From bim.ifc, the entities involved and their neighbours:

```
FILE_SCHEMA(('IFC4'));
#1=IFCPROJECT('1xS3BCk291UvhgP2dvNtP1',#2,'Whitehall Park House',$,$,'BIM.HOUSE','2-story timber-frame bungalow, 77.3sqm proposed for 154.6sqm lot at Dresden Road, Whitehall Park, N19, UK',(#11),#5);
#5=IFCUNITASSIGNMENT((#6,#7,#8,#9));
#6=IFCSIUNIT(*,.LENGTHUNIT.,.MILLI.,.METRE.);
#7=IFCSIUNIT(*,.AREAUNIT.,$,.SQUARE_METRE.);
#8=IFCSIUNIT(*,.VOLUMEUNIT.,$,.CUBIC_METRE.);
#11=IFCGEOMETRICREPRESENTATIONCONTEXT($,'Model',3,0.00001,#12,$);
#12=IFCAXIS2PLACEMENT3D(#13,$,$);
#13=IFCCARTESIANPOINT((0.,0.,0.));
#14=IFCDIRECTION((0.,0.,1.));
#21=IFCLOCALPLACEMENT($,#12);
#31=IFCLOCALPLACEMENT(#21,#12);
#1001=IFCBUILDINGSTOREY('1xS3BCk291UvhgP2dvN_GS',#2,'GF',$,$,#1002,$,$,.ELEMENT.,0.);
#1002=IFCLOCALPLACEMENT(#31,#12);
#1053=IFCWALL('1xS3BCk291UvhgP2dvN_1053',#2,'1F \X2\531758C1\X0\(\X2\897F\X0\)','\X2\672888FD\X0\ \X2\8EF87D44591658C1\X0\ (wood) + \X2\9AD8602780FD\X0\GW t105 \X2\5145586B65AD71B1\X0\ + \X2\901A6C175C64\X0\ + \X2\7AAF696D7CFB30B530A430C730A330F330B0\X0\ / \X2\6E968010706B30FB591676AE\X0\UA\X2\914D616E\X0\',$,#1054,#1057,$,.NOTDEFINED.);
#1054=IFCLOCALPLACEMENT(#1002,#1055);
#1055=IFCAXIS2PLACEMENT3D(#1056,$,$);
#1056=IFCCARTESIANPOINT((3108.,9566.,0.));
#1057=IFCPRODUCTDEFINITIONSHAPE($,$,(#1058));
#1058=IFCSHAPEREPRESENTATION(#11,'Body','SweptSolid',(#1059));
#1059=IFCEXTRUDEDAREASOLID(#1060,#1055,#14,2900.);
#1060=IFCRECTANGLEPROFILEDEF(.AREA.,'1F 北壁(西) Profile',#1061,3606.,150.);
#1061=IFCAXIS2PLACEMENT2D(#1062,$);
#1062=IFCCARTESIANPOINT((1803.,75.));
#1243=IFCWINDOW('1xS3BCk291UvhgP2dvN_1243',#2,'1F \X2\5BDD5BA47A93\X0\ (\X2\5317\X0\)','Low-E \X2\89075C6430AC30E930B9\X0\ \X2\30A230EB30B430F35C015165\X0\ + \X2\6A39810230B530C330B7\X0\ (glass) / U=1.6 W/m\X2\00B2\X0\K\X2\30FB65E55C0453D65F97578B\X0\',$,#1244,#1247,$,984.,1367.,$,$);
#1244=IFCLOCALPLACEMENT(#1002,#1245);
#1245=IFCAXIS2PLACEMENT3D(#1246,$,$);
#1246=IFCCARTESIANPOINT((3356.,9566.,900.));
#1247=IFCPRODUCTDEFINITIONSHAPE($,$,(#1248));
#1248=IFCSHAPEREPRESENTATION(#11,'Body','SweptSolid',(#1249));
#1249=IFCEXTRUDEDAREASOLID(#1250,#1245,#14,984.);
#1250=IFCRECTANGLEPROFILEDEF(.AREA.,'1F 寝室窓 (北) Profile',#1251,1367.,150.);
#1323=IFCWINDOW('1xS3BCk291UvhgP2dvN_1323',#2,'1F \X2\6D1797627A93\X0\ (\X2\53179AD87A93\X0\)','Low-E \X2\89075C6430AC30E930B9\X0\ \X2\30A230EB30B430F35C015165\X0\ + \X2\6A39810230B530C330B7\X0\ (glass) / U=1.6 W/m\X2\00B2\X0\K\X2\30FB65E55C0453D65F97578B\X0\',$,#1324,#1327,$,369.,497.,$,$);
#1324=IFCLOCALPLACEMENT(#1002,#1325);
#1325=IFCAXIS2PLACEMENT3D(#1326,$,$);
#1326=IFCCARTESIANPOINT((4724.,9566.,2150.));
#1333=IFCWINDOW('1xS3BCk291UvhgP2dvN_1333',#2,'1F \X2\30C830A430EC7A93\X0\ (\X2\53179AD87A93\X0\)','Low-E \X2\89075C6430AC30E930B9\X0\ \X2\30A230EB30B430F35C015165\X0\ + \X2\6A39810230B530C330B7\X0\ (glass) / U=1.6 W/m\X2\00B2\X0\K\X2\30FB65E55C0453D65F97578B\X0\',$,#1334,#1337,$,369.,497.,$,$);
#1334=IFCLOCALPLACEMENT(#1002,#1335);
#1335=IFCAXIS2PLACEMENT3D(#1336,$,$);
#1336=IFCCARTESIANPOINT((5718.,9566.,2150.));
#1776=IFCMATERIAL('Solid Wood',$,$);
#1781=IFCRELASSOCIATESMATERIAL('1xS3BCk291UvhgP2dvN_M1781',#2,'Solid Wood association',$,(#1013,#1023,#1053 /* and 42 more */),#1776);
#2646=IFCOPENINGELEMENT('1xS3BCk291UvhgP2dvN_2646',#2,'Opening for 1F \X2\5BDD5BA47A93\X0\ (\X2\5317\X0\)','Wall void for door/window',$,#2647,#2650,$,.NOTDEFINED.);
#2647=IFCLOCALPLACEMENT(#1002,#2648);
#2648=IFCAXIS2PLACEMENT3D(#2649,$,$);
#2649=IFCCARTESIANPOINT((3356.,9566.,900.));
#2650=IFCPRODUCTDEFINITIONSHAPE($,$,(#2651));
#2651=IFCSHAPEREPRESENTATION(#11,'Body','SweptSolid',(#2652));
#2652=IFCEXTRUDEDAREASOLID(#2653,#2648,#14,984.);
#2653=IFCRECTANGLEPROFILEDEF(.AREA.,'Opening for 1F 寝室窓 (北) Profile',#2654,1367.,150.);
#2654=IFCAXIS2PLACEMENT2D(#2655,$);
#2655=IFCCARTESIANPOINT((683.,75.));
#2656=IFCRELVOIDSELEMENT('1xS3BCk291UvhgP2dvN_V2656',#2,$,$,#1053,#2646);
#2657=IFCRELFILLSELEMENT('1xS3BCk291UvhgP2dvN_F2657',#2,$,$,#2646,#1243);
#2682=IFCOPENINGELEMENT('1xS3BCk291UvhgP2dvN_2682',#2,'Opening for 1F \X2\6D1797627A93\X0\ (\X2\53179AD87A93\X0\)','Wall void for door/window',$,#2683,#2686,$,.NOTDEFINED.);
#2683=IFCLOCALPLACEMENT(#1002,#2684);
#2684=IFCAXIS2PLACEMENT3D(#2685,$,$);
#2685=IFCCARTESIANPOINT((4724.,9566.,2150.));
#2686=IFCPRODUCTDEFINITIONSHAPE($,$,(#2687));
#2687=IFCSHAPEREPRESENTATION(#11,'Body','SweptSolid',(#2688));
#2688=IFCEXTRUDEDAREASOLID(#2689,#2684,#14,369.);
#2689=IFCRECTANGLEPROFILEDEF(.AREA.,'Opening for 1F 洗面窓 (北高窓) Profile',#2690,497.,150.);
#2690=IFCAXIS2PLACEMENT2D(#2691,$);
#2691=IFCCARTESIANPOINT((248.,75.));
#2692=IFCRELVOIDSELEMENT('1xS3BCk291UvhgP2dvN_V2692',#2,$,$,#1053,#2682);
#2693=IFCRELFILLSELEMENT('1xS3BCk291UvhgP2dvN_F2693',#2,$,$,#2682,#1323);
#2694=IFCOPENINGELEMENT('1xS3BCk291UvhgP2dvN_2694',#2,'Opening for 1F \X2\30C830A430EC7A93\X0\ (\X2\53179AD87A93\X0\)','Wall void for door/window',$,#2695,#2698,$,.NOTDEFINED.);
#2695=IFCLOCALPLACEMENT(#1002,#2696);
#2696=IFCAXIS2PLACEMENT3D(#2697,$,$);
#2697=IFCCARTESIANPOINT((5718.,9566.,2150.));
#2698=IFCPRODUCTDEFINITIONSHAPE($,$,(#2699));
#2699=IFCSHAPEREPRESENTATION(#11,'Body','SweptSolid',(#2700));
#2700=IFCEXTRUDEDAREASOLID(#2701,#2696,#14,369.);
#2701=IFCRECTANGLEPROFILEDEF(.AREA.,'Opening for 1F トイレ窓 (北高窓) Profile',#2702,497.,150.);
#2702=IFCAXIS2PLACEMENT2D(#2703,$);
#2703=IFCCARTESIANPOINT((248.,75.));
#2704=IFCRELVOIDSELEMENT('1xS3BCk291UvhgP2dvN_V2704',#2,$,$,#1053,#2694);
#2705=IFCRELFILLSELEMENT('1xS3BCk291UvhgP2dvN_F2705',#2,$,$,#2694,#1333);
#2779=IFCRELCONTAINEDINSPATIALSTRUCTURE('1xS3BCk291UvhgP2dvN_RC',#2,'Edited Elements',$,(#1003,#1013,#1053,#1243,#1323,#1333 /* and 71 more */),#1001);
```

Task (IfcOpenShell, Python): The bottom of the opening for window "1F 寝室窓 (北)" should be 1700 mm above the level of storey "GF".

```python
import numpy as np
import ifcopenshell
import ifcopenshell.api.geometry
import ifcopenshell.geom
import ifcopenshell.util.element
import ifcopenshell.util.placement
import ifcopenshell.util.shape
import ifcopenshell.util.unit

model = ifcopenshell.open("bim.ifc")
unit_scale = ifcopenshell.util.unit.calculate_unit_scale(model)

window = model.by_id(1243)
opening = window.FillsVoids[0].RelatingOpeningElement
storey = ifcopenshell.util.element.get_container(window, ifc_class="IfcBuildingStorey")
level = ifcopenshell.util.placement.get_local_placement(storey.ObjectPlacement)[2, 3]

# The opening's origin need not be at the sill, so measure its lowest point.
shape = ifcopenshell.geom.create_shape(ifcopenshell.geom.settings(), opening)
bottom = ifcopenshell.util.shape.get_shape_bottom_elevation(shape, shape.geometry) / unit_scale
dz = level + 1.7 / unit_scale - bottom

shift = np.array([0.0, 0.0, dz])
# The window is not placed relative to its opening, so move both.
for product in (opening, window):
    matrix = ifcopenshell.util.placement.get_local_placement(product.ObjectPlacement)
    matrix[:3, 3] += shift
    ifcopenshell.api.geometry.edit_object_placement(model, product=product, matrix=matrix, is_si=False)

print(f"moved by {dz * unit_scale:+.3f} m")

model.write("bim-out.ifc")
```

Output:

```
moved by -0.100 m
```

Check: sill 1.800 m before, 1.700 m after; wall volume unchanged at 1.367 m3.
